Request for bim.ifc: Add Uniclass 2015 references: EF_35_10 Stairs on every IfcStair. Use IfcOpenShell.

First a look at what the model holds.

```python
import ifcopenshell

model = ifcopenshell.open("bim.ifc")
print(model.schema)
print("classifications:", [c.Name for c in model.by_type("IfcClassification")])
for ifc_class in ("IfcDoor", "IfcRoof", "IfcStair", "IfcWall", "IfcWindow"):
    print(ifc_class, len(model.by_type(ifc_class)))
```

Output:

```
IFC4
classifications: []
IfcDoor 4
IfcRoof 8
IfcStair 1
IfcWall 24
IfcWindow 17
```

```python
import ifcopenshell
import ifcopenshell.api.classification

model = ifcopenshell.open("bim.ifc")

system = ifcopenshell.api.classification.add_classification(model, classification="Uniclass 2015")

codes = {
    "IfcStair": ("EF_35_10", "Stairs"),
}
for ifc_class, (code, name) in codes.items():
    products = model.by_type(ifc_class)
    ifcopenshell.api.classification.add_reference(
        model, products=products, classification=system, identification=code, name=name
    )
    print(code, len(products))

model.write("bim_v2.ifc")
```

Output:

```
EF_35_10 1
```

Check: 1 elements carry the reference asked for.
